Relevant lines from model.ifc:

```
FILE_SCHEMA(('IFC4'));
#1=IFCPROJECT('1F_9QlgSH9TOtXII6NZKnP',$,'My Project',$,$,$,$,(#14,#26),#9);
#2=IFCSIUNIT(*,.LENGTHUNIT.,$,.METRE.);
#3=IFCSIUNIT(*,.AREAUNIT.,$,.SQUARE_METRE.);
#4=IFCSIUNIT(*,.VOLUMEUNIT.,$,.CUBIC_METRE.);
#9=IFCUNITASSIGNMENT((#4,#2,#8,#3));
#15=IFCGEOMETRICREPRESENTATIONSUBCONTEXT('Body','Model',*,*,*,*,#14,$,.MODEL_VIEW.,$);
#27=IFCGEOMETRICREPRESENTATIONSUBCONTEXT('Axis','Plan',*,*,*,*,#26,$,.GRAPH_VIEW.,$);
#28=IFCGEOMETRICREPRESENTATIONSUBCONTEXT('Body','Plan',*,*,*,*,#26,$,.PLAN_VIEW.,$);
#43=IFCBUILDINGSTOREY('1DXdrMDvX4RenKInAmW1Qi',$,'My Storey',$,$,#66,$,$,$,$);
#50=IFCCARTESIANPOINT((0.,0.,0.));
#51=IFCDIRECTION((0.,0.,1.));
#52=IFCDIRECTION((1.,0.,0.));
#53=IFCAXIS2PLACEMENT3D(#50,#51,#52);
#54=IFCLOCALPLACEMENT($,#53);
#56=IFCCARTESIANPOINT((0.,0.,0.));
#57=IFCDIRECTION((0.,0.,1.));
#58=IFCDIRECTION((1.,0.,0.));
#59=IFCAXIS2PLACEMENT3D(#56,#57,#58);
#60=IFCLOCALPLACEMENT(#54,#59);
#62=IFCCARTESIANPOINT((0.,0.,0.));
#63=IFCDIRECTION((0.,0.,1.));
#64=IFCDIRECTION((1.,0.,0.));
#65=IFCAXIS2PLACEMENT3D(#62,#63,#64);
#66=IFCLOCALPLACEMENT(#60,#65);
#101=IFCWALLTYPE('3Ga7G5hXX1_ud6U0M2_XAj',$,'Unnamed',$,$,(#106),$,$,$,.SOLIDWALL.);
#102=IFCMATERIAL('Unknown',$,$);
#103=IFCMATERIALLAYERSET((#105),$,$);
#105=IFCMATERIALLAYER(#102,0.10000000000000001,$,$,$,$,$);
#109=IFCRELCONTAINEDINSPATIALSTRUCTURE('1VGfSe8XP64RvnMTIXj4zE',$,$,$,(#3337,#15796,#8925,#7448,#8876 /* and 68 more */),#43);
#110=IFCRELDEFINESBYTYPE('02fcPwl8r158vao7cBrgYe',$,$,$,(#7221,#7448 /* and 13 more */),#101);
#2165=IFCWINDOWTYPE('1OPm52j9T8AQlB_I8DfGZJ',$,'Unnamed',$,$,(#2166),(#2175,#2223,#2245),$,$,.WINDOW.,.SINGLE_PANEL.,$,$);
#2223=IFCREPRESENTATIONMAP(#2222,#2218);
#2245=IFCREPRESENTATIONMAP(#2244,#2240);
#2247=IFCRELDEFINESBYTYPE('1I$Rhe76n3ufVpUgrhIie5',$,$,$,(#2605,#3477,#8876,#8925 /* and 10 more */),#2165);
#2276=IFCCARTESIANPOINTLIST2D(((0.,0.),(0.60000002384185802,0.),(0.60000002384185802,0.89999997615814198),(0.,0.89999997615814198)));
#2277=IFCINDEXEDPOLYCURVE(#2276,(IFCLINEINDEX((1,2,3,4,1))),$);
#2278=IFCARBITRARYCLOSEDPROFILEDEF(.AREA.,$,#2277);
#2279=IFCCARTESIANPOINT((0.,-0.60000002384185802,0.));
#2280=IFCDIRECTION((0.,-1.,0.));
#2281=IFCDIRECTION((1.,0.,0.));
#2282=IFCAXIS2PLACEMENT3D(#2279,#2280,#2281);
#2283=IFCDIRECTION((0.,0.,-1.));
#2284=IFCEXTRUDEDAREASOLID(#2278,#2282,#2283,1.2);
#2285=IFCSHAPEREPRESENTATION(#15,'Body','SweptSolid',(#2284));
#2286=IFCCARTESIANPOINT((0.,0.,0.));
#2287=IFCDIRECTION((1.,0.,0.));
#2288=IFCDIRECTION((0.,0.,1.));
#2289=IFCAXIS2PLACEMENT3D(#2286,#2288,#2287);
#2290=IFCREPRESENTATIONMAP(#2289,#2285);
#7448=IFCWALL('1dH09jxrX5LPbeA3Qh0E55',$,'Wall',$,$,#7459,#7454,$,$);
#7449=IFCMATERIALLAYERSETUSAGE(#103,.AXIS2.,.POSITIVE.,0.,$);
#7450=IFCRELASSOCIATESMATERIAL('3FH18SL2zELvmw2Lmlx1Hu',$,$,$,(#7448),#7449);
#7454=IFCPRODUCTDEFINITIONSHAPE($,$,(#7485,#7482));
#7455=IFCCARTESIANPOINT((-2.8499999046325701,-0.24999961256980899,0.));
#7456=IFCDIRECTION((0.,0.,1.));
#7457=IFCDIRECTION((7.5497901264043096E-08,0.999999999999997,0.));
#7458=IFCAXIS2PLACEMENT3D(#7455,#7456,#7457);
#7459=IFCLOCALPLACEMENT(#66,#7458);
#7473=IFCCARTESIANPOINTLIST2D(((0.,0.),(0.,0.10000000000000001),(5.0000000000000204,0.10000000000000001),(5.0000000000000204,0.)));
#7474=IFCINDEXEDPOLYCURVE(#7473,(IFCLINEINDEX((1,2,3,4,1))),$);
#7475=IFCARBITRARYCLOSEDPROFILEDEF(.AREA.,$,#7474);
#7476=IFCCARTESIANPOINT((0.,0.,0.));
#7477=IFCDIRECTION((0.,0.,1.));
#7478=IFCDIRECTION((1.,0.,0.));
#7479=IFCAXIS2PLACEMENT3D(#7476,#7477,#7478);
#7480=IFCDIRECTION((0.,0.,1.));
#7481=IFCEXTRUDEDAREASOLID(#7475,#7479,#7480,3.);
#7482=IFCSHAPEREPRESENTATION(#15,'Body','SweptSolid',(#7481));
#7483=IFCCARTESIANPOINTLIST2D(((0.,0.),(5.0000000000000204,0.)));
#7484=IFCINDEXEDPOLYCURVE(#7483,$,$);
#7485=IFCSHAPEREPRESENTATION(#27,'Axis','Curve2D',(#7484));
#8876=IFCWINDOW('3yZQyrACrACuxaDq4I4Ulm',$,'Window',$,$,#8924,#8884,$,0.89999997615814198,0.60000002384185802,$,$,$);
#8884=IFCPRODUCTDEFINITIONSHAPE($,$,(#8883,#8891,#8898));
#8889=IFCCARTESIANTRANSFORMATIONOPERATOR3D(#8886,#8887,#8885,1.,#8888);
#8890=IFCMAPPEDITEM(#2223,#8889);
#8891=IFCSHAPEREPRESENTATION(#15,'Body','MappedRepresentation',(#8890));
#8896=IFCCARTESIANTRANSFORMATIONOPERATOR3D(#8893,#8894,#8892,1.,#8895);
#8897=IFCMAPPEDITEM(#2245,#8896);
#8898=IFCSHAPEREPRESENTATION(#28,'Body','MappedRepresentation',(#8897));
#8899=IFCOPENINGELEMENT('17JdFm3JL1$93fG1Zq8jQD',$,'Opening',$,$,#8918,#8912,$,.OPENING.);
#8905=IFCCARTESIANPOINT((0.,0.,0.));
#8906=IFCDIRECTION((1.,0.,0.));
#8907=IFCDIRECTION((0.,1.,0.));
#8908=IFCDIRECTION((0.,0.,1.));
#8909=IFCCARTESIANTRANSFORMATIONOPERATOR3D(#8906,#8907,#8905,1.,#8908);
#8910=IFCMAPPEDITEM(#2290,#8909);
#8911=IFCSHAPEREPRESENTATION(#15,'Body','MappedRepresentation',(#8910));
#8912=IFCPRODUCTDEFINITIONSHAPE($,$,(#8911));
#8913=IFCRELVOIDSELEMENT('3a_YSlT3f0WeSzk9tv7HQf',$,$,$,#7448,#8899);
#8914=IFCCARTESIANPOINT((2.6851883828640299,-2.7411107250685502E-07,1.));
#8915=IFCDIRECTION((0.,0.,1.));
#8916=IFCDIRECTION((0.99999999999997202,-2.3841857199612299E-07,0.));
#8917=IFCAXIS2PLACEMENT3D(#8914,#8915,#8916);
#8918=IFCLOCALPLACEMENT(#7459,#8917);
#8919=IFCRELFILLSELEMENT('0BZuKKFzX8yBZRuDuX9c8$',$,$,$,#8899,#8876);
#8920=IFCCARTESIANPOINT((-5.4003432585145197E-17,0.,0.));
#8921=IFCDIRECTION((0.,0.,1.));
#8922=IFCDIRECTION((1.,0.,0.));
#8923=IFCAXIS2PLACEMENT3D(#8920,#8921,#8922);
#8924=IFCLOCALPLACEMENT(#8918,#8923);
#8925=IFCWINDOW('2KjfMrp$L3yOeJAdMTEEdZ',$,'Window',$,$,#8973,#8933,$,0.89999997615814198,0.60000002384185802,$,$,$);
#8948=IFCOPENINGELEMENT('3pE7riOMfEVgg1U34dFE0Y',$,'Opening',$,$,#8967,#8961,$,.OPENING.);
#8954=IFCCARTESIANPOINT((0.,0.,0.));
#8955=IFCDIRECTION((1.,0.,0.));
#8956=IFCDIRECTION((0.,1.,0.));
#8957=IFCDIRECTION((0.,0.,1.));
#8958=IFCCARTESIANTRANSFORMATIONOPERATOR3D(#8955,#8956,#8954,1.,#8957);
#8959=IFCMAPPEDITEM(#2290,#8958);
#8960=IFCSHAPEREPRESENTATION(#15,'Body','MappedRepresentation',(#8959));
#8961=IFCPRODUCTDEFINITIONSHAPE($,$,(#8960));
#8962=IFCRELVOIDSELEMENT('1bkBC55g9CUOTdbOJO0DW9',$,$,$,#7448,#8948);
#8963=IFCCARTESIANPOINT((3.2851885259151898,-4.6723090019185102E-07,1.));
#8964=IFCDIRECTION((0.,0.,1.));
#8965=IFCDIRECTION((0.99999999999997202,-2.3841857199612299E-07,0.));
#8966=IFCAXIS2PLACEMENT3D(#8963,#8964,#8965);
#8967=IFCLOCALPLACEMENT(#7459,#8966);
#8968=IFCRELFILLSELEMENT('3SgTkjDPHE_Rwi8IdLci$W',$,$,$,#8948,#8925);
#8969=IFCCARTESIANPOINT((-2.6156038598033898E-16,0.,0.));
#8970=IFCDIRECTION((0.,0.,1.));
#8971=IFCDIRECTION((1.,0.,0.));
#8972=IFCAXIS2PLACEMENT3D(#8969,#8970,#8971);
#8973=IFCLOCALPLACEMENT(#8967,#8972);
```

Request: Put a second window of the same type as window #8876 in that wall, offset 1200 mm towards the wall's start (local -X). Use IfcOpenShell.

```python
import ifcopenshell
import ifcopenshell.api.feature
import ifcopenshell.api.geometry
import ifcopenshell.api.root
import ifcopenshell.geom
import ifcopenshell.util.element
import ifcopenshell.util.placement
import ifcopenshell.util.shape

model = ifcopenshell.open("model.ifc")
settings = ifcopenshell.geom.settings()


def volume(element):
    """Net volume in cubic metres, openings subtracted."""
    shape = ifcopenshell.geom.create_shape(settings, element)
    return ifcopenshell.util.shape.get_volume(shape.geometry)


window = model.by_id(8876)
opening = window.FillsVoids[0].RelatingOpeningElement
wall = opening.VoidsElements[0].RelatingBuildingElement
before = volume(wall)
shift = ifcopenshell.util.placement.get_local_placement(wall.ObjectPlacement)[:3, 0] * -1.2

# copy_class copies the void relationship, type, container and properties, but no geometry.
new_opening = ifcopenshell.api.root.copy_class(model, product=opening)
new_opening.Representation = ifcopenshell.util.element.copy_deep(
    model, opening.Representation, exclude=["IfcGeometricRepresentationContext", "IfcRepresentationMap"]
)
new_window = ifcopenshell.api.root.copy_class(model, product=window)
new_window.Representation = ifcopenshell.util.element.copy_deep(
    model, window.Representation, exclude=["IfcGeometricRepresentationContext", "IfcRepresentationMap"]
)
ifcopenshell.api.feature.add_filling(model, opening=new_opening, element=new_window)

for old, new in ((opening, new_opening), (window, new_window)):
    matrix = ifcopenshell.util.placement.get_local_placement(old.ObjectPlacement)
    matrix[:3, 3] += shift
    ifcopenshell.api.geometry.edit_object_placement(model, product=new, matrix=matrix, is_si=False)

after = volume(wall)

print(f"wall volume {before:.3f} -> {after:.3f} m3")

model.write("model-out.ifc")
```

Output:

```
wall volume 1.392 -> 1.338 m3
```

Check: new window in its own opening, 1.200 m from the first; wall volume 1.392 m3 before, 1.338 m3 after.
